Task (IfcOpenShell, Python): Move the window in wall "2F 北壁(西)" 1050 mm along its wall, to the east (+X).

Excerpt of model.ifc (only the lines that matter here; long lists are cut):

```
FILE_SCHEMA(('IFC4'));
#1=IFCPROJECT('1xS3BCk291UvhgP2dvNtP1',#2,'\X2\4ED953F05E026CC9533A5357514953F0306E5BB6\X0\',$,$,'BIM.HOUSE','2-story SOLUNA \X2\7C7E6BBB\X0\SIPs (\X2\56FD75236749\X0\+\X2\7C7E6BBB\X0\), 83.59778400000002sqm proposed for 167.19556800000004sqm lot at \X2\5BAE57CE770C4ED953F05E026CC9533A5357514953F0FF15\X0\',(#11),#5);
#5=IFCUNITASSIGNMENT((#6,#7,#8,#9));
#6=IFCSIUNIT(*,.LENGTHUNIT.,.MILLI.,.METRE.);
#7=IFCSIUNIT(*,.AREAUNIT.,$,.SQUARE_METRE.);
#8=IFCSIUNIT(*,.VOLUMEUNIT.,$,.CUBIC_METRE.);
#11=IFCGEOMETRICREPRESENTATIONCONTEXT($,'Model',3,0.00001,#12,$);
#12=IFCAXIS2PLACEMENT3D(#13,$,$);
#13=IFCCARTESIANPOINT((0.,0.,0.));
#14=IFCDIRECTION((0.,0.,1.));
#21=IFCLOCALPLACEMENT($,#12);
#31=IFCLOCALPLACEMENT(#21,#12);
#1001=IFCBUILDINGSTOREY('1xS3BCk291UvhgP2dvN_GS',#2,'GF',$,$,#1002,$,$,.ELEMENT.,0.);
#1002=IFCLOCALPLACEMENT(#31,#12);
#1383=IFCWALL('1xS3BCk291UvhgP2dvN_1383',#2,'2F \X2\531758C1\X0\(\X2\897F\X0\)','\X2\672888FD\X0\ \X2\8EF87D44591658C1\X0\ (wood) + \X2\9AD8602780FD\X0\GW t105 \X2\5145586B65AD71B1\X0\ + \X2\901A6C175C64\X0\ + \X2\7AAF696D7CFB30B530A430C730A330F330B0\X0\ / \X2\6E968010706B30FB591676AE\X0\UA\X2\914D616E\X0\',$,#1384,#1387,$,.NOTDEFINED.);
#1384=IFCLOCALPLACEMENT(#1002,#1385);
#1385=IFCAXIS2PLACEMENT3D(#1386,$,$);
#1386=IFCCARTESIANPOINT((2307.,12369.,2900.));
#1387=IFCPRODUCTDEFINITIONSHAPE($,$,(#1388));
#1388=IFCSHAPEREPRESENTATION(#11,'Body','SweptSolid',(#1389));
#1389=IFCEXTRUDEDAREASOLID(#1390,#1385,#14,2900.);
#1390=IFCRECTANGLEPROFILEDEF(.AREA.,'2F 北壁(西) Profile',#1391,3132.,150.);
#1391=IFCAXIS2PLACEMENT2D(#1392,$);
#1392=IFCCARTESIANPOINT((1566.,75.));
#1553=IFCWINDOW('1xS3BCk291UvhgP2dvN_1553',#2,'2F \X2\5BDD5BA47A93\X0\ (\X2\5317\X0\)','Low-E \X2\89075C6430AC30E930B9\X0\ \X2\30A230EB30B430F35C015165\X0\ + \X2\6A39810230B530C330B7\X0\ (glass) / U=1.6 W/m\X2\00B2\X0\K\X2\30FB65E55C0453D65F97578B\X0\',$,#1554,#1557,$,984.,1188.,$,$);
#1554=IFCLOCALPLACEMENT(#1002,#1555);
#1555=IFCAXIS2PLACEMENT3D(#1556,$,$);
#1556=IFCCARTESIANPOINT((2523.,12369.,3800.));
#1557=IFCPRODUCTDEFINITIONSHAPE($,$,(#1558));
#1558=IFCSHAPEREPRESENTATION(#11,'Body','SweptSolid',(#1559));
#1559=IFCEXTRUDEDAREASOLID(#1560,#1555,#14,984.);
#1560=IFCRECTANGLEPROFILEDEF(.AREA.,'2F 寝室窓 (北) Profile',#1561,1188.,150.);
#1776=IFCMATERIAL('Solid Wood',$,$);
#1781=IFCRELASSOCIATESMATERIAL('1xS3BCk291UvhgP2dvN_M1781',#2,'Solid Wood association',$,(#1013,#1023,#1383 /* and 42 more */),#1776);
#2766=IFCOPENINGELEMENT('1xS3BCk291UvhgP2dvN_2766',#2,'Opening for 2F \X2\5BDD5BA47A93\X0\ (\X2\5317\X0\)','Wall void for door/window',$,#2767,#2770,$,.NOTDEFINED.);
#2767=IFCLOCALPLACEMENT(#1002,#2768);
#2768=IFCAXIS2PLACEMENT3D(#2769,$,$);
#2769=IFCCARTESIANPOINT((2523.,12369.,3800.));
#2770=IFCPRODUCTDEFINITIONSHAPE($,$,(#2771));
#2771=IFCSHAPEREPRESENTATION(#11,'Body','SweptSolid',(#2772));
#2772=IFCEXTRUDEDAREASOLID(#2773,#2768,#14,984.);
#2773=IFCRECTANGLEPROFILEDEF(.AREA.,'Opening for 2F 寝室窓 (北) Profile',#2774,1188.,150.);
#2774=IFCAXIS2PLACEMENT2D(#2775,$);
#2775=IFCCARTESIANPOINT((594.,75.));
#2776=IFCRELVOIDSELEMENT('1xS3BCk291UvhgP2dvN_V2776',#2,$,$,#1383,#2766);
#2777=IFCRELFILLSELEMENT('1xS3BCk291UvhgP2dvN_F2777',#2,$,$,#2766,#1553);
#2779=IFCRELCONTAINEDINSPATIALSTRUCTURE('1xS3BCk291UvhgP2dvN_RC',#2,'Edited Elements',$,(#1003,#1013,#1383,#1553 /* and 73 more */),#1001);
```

```python
import ifcopenshell
import ifcopenshell.api.geometry
import ifcopenshell.util.placement
import ifcopenshell.util.unit

model = ifcopenshell.open("model.ifc")
unit_scale = ifcopenshell.util.unit.calculate_unit_scale(model)

window = model.by_guid("1xS3BCk291UvhgP2dvN_1553")
opening = window.FillsVoids[0].RelatingOpeningElement
wall = opening.VoidsElements[0].RelatingBuildingElement

wall_matrix = ifcopenshell.util.placement.get_local_placement(wall.ObjectPlacement)
shift = wall_matrix[:3, 0] * 1.05 / unit_scale
before = ifcopenshell.util.placement.get_local_placement(window.ObjectPlacement)[:3, 3].copy()

# The window is not placed relative to its opening, so move both.
for product in (opening, window):
    matrix = ifcopenshell.util.placement.get_local_placement(product.ObjectPlacement)
    matrix[:3, 3] += shift
    ifcopenshell.api.geometry.edit_object_placement(model, product=product, matrix=matrix, is_si=False)

after = ifcopenshell.util.placement.get_local_placement(window.ObjectPlacement)[:3, 3]
print("window moved by", (after - before).round(3) + 0.0)

model.write("model-out.ifc")
```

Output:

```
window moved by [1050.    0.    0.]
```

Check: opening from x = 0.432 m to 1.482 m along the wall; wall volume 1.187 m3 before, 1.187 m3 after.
